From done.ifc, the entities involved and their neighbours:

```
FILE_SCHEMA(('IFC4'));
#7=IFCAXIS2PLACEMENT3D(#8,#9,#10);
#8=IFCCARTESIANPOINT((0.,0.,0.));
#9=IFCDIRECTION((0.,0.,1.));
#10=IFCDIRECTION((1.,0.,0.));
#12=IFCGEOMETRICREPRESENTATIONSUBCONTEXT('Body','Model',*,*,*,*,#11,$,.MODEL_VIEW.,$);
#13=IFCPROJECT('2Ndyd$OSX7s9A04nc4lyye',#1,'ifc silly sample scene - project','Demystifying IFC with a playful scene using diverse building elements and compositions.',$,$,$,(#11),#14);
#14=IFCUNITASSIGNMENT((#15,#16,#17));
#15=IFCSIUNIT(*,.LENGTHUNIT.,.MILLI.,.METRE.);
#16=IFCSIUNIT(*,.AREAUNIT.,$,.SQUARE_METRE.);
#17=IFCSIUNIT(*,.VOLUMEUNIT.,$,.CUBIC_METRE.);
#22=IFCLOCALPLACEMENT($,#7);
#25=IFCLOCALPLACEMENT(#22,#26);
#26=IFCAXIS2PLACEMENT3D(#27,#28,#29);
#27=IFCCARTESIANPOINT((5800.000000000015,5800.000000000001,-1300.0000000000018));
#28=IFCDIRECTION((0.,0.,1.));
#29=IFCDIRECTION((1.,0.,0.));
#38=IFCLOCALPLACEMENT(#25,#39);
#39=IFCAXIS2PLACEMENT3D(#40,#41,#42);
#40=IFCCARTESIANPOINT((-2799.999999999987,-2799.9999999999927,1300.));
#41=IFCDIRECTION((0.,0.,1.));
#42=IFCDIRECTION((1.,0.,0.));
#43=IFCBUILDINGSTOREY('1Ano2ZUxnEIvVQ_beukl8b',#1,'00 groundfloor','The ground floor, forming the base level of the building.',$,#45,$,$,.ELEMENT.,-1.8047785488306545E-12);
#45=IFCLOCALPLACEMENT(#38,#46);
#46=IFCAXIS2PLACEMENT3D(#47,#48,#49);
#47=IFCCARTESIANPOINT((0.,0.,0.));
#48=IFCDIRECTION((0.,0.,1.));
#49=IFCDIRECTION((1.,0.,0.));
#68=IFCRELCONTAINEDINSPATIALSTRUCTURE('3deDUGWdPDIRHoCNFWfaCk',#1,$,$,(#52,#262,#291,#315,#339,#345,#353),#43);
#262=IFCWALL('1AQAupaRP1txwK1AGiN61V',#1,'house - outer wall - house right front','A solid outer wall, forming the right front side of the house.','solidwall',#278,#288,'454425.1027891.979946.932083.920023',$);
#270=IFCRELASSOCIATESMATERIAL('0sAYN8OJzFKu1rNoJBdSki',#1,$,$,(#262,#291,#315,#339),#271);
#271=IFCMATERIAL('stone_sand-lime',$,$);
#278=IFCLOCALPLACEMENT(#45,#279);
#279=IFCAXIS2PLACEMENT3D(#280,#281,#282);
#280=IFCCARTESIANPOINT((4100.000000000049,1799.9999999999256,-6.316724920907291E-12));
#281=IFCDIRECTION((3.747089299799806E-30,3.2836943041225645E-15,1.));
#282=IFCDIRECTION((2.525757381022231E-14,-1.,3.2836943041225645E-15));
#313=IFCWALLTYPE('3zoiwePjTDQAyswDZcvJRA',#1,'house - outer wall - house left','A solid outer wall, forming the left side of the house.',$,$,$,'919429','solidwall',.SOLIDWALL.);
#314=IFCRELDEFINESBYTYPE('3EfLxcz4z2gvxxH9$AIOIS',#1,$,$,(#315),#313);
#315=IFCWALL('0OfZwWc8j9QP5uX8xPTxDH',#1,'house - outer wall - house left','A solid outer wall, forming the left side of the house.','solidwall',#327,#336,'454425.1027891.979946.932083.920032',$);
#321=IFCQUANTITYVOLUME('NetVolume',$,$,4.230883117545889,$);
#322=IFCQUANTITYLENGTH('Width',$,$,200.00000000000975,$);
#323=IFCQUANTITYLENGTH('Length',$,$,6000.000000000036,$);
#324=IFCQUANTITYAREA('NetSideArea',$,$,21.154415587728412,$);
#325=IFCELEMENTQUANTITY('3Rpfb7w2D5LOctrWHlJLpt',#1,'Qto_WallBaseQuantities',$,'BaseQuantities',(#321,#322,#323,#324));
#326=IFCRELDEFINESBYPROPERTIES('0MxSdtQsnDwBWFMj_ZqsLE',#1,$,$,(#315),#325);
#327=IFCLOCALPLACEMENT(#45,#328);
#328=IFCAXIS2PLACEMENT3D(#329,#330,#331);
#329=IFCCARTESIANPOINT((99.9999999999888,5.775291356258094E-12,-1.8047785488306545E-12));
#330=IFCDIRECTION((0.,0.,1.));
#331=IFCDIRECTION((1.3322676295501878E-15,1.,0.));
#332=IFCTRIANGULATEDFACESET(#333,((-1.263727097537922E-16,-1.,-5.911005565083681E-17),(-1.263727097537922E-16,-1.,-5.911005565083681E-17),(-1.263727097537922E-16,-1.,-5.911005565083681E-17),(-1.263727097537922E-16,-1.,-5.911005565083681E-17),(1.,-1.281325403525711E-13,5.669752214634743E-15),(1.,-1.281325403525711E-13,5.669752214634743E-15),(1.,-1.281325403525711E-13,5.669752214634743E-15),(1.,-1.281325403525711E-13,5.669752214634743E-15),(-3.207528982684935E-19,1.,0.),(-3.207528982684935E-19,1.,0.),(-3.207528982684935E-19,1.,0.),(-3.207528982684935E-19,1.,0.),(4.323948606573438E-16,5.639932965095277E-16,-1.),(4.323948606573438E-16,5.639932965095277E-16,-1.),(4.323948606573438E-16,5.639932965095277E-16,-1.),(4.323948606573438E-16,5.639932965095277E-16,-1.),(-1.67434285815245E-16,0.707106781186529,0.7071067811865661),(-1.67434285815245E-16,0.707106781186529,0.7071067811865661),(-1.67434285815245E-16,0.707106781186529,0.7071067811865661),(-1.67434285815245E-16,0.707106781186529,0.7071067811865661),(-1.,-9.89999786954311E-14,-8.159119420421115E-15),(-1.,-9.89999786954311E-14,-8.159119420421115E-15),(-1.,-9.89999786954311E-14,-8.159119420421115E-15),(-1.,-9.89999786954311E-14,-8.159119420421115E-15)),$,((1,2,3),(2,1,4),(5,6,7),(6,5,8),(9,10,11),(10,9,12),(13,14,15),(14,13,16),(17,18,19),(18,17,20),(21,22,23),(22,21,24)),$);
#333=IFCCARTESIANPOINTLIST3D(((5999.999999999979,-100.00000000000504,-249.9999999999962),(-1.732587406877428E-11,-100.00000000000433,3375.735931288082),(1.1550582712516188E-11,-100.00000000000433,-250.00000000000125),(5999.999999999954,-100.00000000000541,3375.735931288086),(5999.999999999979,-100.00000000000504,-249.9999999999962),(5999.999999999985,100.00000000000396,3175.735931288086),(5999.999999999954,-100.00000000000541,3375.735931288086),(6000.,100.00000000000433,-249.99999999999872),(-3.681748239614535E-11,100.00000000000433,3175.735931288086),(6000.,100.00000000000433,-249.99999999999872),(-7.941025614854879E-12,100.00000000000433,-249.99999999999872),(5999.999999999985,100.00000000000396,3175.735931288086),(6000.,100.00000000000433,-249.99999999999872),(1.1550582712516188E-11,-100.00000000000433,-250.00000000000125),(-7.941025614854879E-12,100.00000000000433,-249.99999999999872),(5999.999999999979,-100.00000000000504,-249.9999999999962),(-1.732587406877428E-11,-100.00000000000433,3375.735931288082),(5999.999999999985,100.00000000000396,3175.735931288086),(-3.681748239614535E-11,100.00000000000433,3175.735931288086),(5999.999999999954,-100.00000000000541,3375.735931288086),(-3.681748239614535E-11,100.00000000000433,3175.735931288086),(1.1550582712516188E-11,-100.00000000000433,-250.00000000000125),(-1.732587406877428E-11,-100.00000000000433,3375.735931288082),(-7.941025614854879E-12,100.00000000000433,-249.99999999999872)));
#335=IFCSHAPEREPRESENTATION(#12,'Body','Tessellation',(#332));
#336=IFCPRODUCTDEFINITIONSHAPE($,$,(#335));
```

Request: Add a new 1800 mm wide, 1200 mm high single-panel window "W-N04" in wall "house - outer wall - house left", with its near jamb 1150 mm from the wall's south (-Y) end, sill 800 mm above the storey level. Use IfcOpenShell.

```python
import numpy as np
import ifcopenshell
import ifcopenshell.api.feature
import ifcopenshell.api.geometry
import ifcopenshell.api.pset
import ifcopenshell.api.root
import ifcopenshell.api.spatial
import ifcopenshell.geom
import ifcopenshell.util.element
import ifcopenshell.util.placement
import ifcopenshell.util.representation
import ifcopenshell.util.shape
import ifcopenshell.util.unit

model = ifcopenshell.open("done.ifc")
unit_scale = ifcopenshell.util.unit.calculate_unit_scale(model)
area_scale = ifcopenshell.util.unit.calculate_unit_scale(model, "AREAUNIT")
volume_scale = ifcopenshell.util.unit.calculate_unit_scale(model, "VOLUMEUNIT")
settings = ifcopenshell.geom.settings()


def volume(element):
    """Net volume in cubic metres, openings subtracted."""
    shape = ifcopenshell.geom.create_shape(settings, element)
    return ifcopenshell.util.shape.get_volume(shape.geometry)


wall = model.by_guid("0OfZwWc8j9QP5uX8xPTxDH")
storey = ifcopenshell.util.element.get_container(wall, ifc_class="IfcBuildingStorey")
context = ifcopenshell.util.representation.get_context(model, "Model", "Body", "MODEL_VIEW")
before = volume(wall)

width, height, from_end, sill = 1.8, 1.2, 1.15, 0.8  # metres

# The wall runs along its own X axis, and the end named is its -X end.
wall_shape = ifcopenshell.geom.create_shape(settings, wall)
x, y, z = ifcopenshell.util.shape.get_vertices(wall_shape.geometry).T
start = x.min() + from_end
face, thickness = float(y.min()), float(y.max() - y.min())
wall_matrix = ifcopenshell.util.placement.get_local_placement(wall.ObjectPlacement)
level = ifcopenshell.util.placement.get_local_placement(storey.ObjectPlacement)[2, 3]


def in_wall(x, y):
    """Placement at x, y metres in the wall's axes, at sill height."""
    matrix = wall_matrix.copy()
    matrix[:, 3] = wall_matrix @ np.array([x / unit_scale, y / unit_scale, 0.0, 1.0])
    matrix[2, 3] = level + sill / unit_scale
    return matrix


# Opening: a box that overshoots both wall faces by 50 mm.
opening = ifcopenshell.api.root.create_entity(model, ifc_class="IfcOpeningElement", predefined_type="OPENING")
box = ifcopenshell.api.geometry.add_wall_representation(
    model, context=context, length=width, height=height, thickness=thickness + 0.1
)
ifcopenshell.api.geometry.assign_representation(model, product=opening, representation=box)
ifcopenshell.api.geometry.edit_object_placement(model, product=opening, matrix=in_wall(start, face - 0.05), is_si=False)
ifcopenshell.api.feature.add_feature(model, feature=opening, element=wall)

window = ifcopenshell.api.root.create_entity(model, ifc_class="IfcWindow", name="W-N04", predefined_type="WINDOW")
window.OverallWidth, window.OverallHeight = width / unit_scale, height / unit_scale
window.PartitioningType = "SINGLE_PANEL"
body = ifcopenshell.api.geometry.add_window_representation(
    model,
    context=context,
    overall_width=window.OverallWidth,
    overall_height=window.OverallHeight,
    partition_type="SINGLE_PANEL",
)
ifcopenshell.api.geometry.assign_representation(model, product=window, representation=body)
ifcopenshell.api.spatial.assign_container(model, products=[window], relating_structure=storey)
ifcopenshell.api.feature.add_filling(model, opening=opening, element=window)

# Centre the window in the wall's thickness.
ifcopenshell.api.geometry.edit_object_placement(model, product=window, matrix=in_wall(start, face), is_si=False)
window_shape = ifcopenshell.geom.create_shape(settings, window)
depth = ifcopenshell.util.shape.get_vertices(window_shape.geometry)[:, 1]
offset = face + thickness / 2 - (depth.min() + depth.max()) / 2
ifcopenshell.api.geometry.edit_object_placement(model, product=window, matrix=in_wall(start, offset), is_si=False)

after = volume(wall)

# Update the wall's stored quantities.
qto = model.by_id(ifcopenshell.util.element.get_pset(wall, "Qto_WallBaseQuantities", should_inherit=False)["id"])
ifcopenshell.api.pset.edit_qto(model, qto=qto, properties={
    "NetVolume": after / volume_scale,
    "NetSideArea": after / thickness / area_scale,
})

print(f"wall volume {before:.3f} -> {after:.3f} m3")

model.write("done_updated.ifc")
```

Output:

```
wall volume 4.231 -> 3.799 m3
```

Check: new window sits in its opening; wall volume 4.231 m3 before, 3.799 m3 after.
